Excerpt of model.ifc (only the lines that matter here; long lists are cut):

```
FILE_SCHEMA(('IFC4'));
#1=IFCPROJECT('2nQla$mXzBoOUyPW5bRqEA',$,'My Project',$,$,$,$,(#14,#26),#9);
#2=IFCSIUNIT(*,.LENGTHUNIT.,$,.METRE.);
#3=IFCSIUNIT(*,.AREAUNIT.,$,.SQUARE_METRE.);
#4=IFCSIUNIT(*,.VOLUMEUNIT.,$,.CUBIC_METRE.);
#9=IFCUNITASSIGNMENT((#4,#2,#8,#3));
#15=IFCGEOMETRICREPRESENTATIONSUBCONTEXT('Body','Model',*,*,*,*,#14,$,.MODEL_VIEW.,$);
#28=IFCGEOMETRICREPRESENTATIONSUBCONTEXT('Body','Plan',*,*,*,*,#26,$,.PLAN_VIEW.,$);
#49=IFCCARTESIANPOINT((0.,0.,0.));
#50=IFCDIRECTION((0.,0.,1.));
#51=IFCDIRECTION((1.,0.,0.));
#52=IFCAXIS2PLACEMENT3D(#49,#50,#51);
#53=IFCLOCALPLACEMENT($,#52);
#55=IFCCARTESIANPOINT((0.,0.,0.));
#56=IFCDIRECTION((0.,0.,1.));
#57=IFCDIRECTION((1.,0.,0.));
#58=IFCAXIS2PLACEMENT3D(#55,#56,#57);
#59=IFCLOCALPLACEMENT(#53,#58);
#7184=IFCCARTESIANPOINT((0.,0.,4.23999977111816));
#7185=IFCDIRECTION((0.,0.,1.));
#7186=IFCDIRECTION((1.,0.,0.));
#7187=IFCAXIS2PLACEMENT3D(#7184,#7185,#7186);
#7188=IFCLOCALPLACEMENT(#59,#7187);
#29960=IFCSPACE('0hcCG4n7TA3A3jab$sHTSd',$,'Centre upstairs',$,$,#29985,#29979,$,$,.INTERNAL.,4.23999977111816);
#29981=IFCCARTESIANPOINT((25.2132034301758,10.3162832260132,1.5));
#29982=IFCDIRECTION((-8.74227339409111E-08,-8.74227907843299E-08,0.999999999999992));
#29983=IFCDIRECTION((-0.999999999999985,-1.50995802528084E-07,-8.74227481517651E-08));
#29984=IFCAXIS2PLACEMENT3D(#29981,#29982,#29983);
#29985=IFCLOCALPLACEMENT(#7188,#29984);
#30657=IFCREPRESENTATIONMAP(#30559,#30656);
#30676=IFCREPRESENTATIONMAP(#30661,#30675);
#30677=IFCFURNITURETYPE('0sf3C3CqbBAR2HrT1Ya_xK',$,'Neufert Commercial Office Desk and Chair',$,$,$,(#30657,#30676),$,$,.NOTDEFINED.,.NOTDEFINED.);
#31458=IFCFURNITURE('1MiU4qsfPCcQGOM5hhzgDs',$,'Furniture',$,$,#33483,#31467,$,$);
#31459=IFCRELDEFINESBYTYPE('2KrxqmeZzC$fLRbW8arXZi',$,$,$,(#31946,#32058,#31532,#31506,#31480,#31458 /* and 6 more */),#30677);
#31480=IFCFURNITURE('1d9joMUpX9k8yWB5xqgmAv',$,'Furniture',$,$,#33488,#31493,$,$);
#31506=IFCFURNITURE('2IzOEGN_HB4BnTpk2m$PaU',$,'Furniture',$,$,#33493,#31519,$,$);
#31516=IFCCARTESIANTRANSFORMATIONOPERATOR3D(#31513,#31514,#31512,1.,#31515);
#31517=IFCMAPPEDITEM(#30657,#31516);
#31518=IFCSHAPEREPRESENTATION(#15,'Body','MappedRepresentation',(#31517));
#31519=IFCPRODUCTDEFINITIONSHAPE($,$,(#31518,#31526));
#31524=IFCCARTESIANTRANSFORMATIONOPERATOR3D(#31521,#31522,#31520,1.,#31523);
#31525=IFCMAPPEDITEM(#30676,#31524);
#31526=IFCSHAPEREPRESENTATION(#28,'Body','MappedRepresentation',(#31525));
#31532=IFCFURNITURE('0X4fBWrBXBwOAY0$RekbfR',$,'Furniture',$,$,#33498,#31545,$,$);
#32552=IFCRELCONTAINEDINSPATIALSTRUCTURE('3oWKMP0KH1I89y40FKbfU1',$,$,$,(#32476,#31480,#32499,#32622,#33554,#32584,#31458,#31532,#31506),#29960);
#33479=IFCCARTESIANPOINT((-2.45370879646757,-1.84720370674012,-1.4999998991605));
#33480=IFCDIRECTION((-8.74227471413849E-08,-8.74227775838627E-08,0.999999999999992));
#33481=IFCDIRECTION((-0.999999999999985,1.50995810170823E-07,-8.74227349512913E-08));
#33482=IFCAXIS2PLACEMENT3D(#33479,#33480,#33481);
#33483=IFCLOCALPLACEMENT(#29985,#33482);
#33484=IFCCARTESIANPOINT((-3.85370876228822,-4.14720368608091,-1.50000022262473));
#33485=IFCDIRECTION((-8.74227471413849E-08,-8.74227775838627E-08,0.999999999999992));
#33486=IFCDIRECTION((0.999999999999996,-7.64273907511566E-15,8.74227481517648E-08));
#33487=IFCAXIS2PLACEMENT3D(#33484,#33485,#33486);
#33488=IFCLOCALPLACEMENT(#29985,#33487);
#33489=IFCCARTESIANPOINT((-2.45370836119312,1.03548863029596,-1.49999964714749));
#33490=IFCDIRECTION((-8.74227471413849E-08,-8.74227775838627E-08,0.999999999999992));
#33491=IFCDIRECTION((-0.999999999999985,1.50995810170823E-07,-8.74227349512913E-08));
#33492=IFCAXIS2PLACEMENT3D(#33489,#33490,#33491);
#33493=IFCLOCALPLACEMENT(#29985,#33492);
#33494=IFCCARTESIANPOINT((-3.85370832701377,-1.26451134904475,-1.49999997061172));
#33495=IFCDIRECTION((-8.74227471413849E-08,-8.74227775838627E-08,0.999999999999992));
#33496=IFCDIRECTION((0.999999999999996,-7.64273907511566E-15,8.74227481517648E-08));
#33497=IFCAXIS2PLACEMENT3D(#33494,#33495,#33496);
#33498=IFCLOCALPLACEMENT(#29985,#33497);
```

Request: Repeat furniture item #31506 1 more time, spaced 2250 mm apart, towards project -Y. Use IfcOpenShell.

```python
import numpy as np
import ifcopenshell
import ifcopenshell.api.geometry
import ifcopenshell.api.root
import ifcopenshell.util.element
import ifcopenshell.util.placement

model = ifcopenshell.open("model.ifc")

source = model.by_guid("2IzOEGN_HB4BnTpk2m$PaU")
base = ifcopenshell.util.placement.get_local_placement(source.ObjectPlacement)
step = np.array([0.0, -1.0, 0.0]) * 2.25

for i in range(1, 2):
    copy = ifcopenshell.api.root.copy_class(model, product=source)
    copy.Representation = ifcopenshell.util.element.copy_deep(
        model, source.Representation, exclude=["IfcGeometricRepresentationContext", "IfcRepresentationMap"]
    )
    matrix = base.copy()
    matrix[:3, 3] += i * step
    print("added at", matrix[:3, 3].round(3) + 0.0)
    ifcopenshell.api.geometry.edit_object_placement(model, product=copy, matrix=matrix, is_si=False)

model.write("model_updated.ifc")
```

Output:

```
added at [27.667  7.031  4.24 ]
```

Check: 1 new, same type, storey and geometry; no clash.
